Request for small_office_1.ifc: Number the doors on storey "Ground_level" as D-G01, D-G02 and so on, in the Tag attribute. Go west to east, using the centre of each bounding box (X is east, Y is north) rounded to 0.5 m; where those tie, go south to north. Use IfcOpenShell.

First a look at what the model holds.

```python
import ifcopenshell
import ifcopenshell.util.element
import ifcopenshell.util.placement

model = ifcopenshell.open("small_office_1.ifc")
print(model.schema)
storey = next(s for s in model.by_type("IfcBuildingStorey") if s.Name == "Ground_level")
doors = [e for e in ifcopenshell.util.element.get_decomposition(storey) if e.is_a("IfcDoor")]
for e in sorted(doors, key=lambda e: e.id()):
    origin = ifcopenshell.util.placement.get_local_placement(e.ObjectPlacement)[:3, 3]
    print(e.id(), e.Tag, e.Name, origin.round(2) + 0.0, sep=" | ")
```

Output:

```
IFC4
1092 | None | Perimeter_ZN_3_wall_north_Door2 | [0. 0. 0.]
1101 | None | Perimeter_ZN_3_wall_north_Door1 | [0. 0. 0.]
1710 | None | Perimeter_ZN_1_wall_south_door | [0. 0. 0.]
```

```python
import ifcopenshell
import ifcopenshell.geom
import ifcopenshell.util.element
import ifcopenshell.util.shape

model = ifcopenshell.open("small_office_1.ifc")
settings = ifcopenshell.geom.settings()
settings.set("use-world-coords", True)


def centre(element):
    shape = ifcopenshell.geom.create_shape(settings, element)
    return ifcopenshell.util.shape.get_bbox_centroid(shape.geometry)


storey = next(s for s in model.by_type("IfcBuildingStorey") if s.Name == "Ground_level")
doors = [e for e in ifcopenshell.util.element.get_decomposition(storey) if e.is_a("IfcDoor")]

# Insertion points can sit at a corner or the storey origin, so sort by the geometry (in metres).
centres = {e: centre(e) for e in doors}
doors.sort(key=lambda e: (round(centres[e][0] / 0.5), centres[e][1]))

for i, e in enumerate(doors, start=1):
    number = f"D-G{i:02d}"
    e.Tag = number
    print(e.id(), number)

model.write("small_office_1_v2.ifc")
```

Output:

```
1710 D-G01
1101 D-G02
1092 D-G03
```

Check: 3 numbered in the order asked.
